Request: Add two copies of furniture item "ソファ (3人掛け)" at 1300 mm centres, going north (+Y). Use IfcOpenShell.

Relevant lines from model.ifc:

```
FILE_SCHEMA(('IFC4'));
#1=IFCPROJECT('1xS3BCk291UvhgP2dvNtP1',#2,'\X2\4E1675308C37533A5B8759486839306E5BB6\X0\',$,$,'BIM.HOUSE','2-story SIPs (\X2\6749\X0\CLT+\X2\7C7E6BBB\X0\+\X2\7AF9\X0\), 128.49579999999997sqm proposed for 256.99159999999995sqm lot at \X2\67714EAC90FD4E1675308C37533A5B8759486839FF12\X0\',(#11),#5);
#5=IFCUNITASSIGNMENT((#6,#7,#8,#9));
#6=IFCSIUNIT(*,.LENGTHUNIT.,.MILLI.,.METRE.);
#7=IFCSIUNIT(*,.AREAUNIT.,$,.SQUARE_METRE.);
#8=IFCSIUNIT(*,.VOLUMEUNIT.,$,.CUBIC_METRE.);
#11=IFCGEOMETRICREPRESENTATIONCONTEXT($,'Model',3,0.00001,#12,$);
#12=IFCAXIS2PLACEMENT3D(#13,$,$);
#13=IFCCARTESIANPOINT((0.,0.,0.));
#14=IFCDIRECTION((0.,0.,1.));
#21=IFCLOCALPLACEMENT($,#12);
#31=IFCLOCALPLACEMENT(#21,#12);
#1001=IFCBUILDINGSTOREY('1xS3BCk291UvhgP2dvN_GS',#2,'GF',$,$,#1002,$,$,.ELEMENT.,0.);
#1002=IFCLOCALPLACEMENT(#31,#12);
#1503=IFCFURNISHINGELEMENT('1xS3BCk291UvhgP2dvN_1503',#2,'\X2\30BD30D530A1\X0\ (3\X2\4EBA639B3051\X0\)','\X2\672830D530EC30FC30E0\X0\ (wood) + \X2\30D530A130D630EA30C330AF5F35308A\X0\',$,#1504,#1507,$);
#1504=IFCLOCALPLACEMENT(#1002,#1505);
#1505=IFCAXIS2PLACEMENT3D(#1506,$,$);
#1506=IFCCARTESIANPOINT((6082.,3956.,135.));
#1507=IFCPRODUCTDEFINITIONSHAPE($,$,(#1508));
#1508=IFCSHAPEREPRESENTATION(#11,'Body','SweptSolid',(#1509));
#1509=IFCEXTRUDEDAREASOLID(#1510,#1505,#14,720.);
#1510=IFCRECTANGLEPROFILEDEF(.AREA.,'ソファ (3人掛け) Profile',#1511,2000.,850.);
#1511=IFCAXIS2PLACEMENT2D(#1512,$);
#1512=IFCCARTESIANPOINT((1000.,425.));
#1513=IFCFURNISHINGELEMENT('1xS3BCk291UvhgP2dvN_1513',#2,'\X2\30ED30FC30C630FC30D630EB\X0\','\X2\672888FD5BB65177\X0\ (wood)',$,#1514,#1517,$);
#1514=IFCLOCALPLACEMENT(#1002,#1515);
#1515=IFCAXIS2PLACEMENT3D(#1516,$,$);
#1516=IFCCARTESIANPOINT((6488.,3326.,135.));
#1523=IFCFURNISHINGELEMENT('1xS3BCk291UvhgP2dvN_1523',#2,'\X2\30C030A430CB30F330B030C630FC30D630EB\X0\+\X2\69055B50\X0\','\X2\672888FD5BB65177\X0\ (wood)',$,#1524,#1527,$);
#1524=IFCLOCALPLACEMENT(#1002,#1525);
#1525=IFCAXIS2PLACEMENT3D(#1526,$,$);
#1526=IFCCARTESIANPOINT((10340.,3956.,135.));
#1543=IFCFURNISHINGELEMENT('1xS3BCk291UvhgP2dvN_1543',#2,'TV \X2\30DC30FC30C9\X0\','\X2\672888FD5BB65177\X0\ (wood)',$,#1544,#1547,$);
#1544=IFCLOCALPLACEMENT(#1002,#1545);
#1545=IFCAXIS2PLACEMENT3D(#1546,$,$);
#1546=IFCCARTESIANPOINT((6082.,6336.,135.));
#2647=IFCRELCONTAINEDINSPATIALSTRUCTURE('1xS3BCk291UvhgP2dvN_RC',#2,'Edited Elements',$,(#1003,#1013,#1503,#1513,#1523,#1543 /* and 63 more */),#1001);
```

```python
import numpy as np
import ifcopenshell
import ifcopenshell.api.geometry
import ifcopenshell.api.root
import ifcopenshell.util.element
import ifcopenshell.util.placement
import ifcopenshell.util.unit

model = ifcopenshell.open("model.ifc")
unit_scale = ifcopenshell.util.unit.calculate_unit_scale(model)


def reuse_history(source, copy):
    """copy_class also copies each property set's owner history, people and application; keep the originals."""
    for rel in copy.IsDefinedBy:
        if rel.is_a("IfcRelDefinesByProperties") and (history := rel.RelatingPropertyDefinition.OwnerHistory):
            rel.RelatingPropertyDefinition.OwnerHistory = source.OwnerHistory
            ifcopenshell.util.element.remove_deep2(model, history)


source = model.by_guid("1xS3BCk291UvhgP2dvN_1503")
base = ifcopenshell.util.placement.get_local_placement(source.ObjectPlacement)
step = np.array([0.0, 1.0, 0.0]) * 1.3 / unit_scale

for i in range(1, 3):
    copy = ifcopenshell.api.root.copy_class(model, product=source)
    copy.Representation = ifcopenshell.util.element.copy_deep(
        model, source.Representation, exclude=["IfcGeometricRepresentationContext", "IfcRepresentationMap"]
    )
    reuse_history(source, copy)
    matrix = base.copy()
    matrix[:3, 3] += i * step
    print("added at", matrix[:3, 3].round(3) + 0.0)
    ifcopenshell.api.geometry.edit_object_placement(model, product=copy, matrix=matrix, is_si=False)

model.write("model_v2.ifc")
```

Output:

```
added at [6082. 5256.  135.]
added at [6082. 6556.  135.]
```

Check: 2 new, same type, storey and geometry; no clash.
